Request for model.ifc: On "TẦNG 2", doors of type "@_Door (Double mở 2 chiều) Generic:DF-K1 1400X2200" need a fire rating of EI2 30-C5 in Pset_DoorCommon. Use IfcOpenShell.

First a look at what the model holds.

```python
import ifcopenshell
import ifcopenshell.util.element

model = ifcopenshell.open("model.ifc")
print(model.schema)
storey = next(s for s in model.by_type("IfcBuildingStorey") if s.Name == "TẦNG 2")
doors = [e for e in ifcopenshell.util.element.get_decomposition(storey) if e.is_a("IfcDoor")]
seen = {}
for e in doors:
    element_type = ifcopenshell.util.element.get_type(e)
    key = (element_type.Name if element_type != e and element_type else None, ifcopenshell.util.element.get_pset(e, "Pset_DoorCommon", "FireRating"))
    seen[key] = seen.get(key, 0) + 1
for (name, value), count in sorted(seen.items(), key=str):
    print(count, "x", name, "|", value)
```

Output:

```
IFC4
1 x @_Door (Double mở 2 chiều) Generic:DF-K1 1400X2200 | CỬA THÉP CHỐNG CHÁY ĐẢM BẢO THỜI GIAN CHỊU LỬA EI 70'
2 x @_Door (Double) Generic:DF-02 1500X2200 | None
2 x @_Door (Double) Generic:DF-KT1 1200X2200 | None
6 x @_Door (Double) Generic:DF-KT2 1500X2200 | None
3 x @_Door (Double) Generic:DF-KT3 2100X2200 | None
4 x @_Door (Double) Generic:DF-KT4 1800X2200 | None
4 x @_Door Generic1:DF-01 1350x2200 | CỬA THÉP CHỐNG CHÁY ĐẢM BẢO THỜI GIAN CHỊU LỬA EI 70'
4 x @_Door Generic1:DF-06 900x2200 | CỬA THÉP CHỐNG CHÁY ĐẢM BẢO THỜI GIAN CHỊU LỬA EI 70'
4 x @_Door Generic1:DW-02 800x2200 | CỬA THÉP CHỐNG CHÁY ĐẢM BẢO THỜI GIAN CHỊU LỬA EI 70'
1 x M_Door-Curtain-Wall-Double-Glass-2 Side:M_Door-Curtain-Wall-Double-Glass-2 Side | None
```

```python
import ifcopenshell
import ifcopenshell.api.pset
import ifcopenshell.util.element

model = ifcopenshell.open("model.ifc")

storey = next(s for s in model.by_type("IfcBuildingStorey") if s.Name == "TẦNG 2")
doors = [e for e in ifcopenshell.util.element.get_decomposition(storey) if e.is_a("IfcDoor")]

count = 0
for e in doors:
    element_type = ifcopenshell.util.element.get_type(e)
    if element_type in (None, e) or element_type.Name != "@_Door (Double mở 2 chiều) Generic:DF-K1 1400X2200":
        continue
    # add_pset returns the element's existing set when there is one.
    pset = ifcopenshell.api.pset.add_pset(model, product=e, name="Pset_DoorCommon")
    ifcopenshell.api.pset.edit_pset(model, pset=pset, properties={"FireRating": "EI2 30-C5"})
    count += 1

print(count, "doors updated")

model.write("model-out.ifc")
```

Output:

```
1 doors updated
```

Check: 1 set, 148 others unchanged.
